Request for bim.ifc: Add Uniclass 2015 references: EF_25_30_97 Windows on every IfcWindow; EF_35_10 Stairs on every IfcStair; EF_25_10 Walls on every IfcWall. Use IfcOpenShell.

First a look at what the model holds.

```python
import ifcopenshell

model = ifcopenshell.open("bim.ifc")
print(model.schema)
print("classifications:", [c.Name for c in model.by_type("IfcClassification")])
for ifc_class in ("IfcDoor", "IfcRoof", "IfcStair", "IfcWall", "IfcWindow"):
    print(ifc_class, len(model.by_type(ifc_class)))
```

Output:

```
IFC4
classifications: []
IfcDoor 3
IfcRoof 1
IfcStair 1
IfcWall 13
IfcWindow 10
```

```python
import ifcopenshell
import ifcopenshell.api.classification

model = ifcopenshell.open("bim.ifc")

system = ifcopenshell.api.classification.add_classification(model, classification="Uniclass 2015")

codes = {
    "IfcWindow": ("EF_25_30_97", "Windows"),
    "IfcStair": ("EF_35_10", "Stairs"),
    "IfcWall": ("EF_25_10", "Walls"),
}
for ifc_class, (code, name) in codes.items():
    products = model.by_type(ifc_class)
    ifcopenshell.api.classification.add_reference(
        model, products=products, classification=system, identification=code, name=name
    )
    print(code, len(products))

model.write("bim-out.ifc")
```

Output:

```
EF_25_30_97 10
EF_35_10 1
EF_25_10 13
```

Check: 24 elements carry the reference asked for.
